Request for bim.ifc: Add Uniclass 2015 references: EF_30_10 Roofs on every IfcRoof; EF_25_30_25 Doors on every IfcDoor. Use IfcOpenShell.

First a look at what the model holds.

```python
import ifcopenshell

model = ifcopenshell.open("bim.ifc")
print(model.schema)
print("classifications:", [c.Name for c in model.by_type("IfcClassification")])
for ifc_class in ("IfcDoor", "IfcRoof", "IfcStair", "IfcWall", "IfcWindow"):
    print(ifc_class, len(model.by_type(ifc_class)))
```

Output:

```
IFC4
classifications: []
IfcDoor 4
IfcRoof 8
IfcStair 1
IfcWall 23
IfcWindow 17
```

```python
import ifcopenshell
import ifcopenshell.api.classification

model = ifcopenshell.open("bim.ifc")

system = ifcopenshell.api.classification.add_classification(model, classification="Uniclass 2015")

codes = {
    "IfcRoof": ("EF_30_10", "Roofs"),
    "IfcDoor": ("EF_25_30_25", "Doors"),
}
for ifc_class, (code, name) in codes.items():
    products = model.by_type(ifc_class)
    ifcopenshell.api.classification.add_reference(
        model, products=products, classification=system, identification=code, name=name
    )
    print(code, len(products))

model.write("bim_updated.ifc")
```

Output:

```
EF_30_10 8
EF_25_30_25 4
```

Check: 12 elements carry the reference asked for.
